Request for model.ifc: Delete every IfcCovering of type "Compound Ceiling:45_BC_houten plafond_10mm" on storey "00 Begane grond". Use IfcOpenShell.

First a look at what the model holds.

```python
import ifcopenshell
import ifcopenshell.util.element

model = ifcopenshell.open("model.ifc")
print(model.schema)
storey = next(s for s in model.by_type("IfcBuildingStorey") if s.Name == "00 Begane grond")
coverings = [e for e in ifcopenshell.util.element.get_decomposition(storey) if e.is_a("IfcCovering")]
seen = {}
for e in coverings:
    element_type = ifcopenshell.util.element.get_type(e)
    name = element_type.Name if element_type not in (None, e) else None
    seen[name] = seen.get(name, 0) + 1
for name, count in sorted(seen.items(), key=str):
    print(count, "x", name)
```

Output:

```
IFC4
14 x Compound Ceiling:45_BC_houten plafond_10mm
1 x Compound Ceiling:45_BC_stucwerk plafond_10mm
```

```python
import ifcopenshell
import ifcopenshell.api.root
import ifcopenshell.util.element

model = ifcopenshell.open("model.ifc")

storey = next(s for s in model.by_type("IfcBuildingStorey") if s.Name == "00 Begane grond")
coverings = [e for e in ifcopenshell.util.element.get_decomposition(storey) if e.is_a("IfcCovering")]
targets = [e for e in coverings if (t := ifcopenshell.util.element.get_type(e)) not in (None, e) and t.Name == "Compound Ceiling:45_BC_houten plafond_10mm"]

for e in targets:
    ifcopenshell.api.root.remove_product(model, product=e)
print(len(targets), "removed")

model.write("model_v2.ifc")
```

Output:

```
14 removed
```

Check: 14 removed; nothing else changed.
